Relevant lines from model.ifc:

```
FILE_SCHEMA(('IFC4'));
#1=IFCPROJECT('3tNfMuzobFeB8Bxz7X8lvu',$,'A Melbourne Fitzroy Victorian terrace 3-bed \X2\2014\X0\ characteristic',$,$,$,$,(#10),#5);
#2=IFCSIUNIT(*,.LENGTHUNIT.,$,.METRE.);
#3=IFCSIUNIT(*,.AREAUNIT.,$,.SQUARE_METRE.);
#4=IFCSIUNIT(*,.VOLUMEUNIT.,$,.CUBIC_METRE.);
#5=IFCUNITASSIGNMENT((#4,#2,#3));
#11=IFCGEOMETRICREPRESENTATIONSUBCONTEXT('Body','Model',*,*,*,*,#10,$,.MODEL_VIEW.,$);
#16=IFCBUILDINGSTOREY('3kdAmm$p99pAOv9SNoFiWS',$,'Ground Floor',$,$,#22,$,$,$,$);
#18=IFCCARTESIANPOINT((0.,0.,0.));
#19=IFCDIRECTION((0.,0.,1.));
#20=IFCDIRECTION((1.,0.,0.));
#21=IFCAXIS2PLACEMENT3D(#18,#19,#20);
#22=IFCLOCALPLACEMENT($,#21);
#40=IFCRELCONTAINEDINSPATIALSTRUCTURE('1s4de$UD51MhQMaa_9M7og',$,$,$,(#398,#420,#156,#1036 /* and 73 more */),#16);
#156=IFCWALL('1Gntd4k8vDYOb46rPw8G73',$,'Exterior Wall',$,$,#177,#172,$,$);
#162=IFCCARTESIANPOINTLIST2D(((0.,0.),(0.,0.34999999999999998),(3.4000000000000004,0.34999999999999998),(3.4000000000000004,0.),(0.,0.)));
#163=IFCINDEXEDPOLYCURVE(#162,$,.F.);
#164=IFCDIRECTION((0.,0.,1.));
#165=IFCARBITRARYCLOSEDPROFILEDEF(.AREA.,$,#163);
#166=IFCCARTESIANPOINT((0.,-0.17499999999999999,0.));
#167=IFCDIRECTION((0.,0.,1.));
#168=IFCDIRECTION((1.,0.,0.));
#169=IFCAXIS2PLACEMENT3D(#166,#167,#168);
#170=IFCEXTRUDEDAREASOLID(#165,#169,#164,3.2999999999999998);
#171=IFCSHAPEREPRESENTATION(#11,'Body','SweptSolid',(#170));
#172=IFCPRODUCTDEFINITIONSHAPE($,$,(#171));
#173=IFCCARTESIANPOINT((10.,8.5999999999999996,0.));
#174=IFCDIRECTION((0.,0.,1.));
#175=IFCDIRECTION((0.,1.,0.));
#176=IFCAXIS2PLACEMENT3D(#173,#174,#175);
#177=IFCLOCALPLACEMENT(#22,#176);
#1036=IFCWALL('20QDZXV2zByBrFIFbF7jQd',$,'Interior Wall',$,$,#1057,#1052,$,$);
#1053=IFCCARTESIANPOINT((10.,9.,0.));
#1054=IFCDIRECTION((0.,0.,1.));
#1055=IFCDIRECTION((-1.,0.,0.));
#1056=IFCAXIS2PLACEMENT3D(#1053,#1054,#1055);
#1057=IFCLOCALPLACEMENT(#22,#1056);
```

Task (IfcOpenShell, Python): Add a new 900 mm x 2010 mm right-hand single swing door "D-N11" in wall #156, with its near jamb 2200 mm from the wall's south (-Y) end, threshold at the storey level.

```python
import numpy as np
import ifcopenshell
import ifcopenshell.api.feature
import ifcopenshell.api.geometry
import ifcopenshell.api.root
import ifcopenshell.api.spatial
import ifcopenshell.geom
import ifcopenshell.util.element
import ifcopenshell.util.placement
import ifcopenshell.util.representation
import ifcopenshell.util.shape
import ifcopenshell.util.unit

model = ifcopenshell.open("model.ifc")
unit_scale = ifcopenshell.util.unit.calculate_unit_scale(model)
settings = ifcopenshell.geom.settings()


def volume(element):
    """Net volume in cubic metres, openings subtracted."""
    shape = ifcopenshell.geom.create_shape(settings, element)
    return ifcopenshell.util.shape.get_volume(shape.geometry)


wall = model.by_guid("1Gntd4k8vDYOb46rPw8G73")
storey = ifcopenshell.util.element.get_container(wall, ifc_class="IfcBuildingStorey")
context = ifcopenshell.util.representation.get_context(model, "Model", "Body", "MODEL_VIEW")
before = volume(wall)

width, height, from_end, sill = 0.9, 2.01, 2.2, 0.0  # metres

# The wall runs along its own X axis, and the end named is its -X end.
wall_shape = ifcopenshell.geom.create_shape(settings, wall)
x, y, z = ifcopenshell.util.shape.get_vertices(wall_shape.geometry).T
start = x.min() + from_end
face, thickness = float(y.min()), float(y.max() - y.min())
wall_matrix = ifcopenshell.util.placement.get_local_placement(wall.ObjectPlacement)
level = ifcopenshell.util.placement.get_local_placement(storey.ObjectPlacement)[2, 3]


def in_wall(x, y):
    """Placement at x, y metres in the wall's axes, at sill height."""
    matrix = wall_matrix.copy()
    matrix[:, 3] = wall_matrix @ np.array([x / unit_scale, y / unit_scale, 0.0, 1.0])
    matrix[2, 3] = level + sill / unit_scale
    return matrix


# Opening: a box that overshoots both wall faces by 50 mm.
opening = ifcopenshell.api.root.create_entity(model, ifc_class="IfcOpeningElement", predefined_type="OPENING")
box = ifcopenshell.api.geometry.add_wall_representation(
    model, context=context, length=width, height=height, thickness=thickness + 0.1
)
ifcopenshell.api.geometry.assign_representation(model, product=opening, representation=box)
ifcopenshell.api.geometry.edit_object_placement(model, product=opening, matrix=in_wall(start, face - 0.05), is_si=False)
ifcopenshell.api.feature.add_feature(model, feature=opening, element=wall)

door = ifcopenshell.api.root.create_entity(model, ifc_class="IfcDoor", name="D-N11", predefined_type="DOOR")
door.OverallWidth, door.OverallHeight = width / unit_scale, height / unit_scale
door.OperationType = "SINGLE_SWING_RIGHT"
body = ifcopenshell.api.geometry.add_door_representation(
    model,
    context=context,
    overall_width=door.OverallWidth,
    overall_height=door.OverallHeight,
    operation_type="SINGLE_SWING_RIGHT",
    lining_properties={"LiningDepth": thickness / unit_scale, "ThresholdDepth": thickness / unit_scale},
)
ifcopenshell.api.geometry.assign_representation(model, product=door, representation=body)
ifcopenshell.api.spatial.assign_container(model, products=[door], relating_structure=storey)
ifcopenshell.api.feature.add_filling(model, opening=opening, element=door)

# The lining spans the wall, so the door starts at the wall face.
ifcopenshell.api.geometry.edit_object_placement(model, product=door, matrix=in_wall(start, face), is_si=False)

after = volume(wall)

print(f"wall volume {before:.3f} -> {after:.3f} m3")

model.write("model-out.ifc")
```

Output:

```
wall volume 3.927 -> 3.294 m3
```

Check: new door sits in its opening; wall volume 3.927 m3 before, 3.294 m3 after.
